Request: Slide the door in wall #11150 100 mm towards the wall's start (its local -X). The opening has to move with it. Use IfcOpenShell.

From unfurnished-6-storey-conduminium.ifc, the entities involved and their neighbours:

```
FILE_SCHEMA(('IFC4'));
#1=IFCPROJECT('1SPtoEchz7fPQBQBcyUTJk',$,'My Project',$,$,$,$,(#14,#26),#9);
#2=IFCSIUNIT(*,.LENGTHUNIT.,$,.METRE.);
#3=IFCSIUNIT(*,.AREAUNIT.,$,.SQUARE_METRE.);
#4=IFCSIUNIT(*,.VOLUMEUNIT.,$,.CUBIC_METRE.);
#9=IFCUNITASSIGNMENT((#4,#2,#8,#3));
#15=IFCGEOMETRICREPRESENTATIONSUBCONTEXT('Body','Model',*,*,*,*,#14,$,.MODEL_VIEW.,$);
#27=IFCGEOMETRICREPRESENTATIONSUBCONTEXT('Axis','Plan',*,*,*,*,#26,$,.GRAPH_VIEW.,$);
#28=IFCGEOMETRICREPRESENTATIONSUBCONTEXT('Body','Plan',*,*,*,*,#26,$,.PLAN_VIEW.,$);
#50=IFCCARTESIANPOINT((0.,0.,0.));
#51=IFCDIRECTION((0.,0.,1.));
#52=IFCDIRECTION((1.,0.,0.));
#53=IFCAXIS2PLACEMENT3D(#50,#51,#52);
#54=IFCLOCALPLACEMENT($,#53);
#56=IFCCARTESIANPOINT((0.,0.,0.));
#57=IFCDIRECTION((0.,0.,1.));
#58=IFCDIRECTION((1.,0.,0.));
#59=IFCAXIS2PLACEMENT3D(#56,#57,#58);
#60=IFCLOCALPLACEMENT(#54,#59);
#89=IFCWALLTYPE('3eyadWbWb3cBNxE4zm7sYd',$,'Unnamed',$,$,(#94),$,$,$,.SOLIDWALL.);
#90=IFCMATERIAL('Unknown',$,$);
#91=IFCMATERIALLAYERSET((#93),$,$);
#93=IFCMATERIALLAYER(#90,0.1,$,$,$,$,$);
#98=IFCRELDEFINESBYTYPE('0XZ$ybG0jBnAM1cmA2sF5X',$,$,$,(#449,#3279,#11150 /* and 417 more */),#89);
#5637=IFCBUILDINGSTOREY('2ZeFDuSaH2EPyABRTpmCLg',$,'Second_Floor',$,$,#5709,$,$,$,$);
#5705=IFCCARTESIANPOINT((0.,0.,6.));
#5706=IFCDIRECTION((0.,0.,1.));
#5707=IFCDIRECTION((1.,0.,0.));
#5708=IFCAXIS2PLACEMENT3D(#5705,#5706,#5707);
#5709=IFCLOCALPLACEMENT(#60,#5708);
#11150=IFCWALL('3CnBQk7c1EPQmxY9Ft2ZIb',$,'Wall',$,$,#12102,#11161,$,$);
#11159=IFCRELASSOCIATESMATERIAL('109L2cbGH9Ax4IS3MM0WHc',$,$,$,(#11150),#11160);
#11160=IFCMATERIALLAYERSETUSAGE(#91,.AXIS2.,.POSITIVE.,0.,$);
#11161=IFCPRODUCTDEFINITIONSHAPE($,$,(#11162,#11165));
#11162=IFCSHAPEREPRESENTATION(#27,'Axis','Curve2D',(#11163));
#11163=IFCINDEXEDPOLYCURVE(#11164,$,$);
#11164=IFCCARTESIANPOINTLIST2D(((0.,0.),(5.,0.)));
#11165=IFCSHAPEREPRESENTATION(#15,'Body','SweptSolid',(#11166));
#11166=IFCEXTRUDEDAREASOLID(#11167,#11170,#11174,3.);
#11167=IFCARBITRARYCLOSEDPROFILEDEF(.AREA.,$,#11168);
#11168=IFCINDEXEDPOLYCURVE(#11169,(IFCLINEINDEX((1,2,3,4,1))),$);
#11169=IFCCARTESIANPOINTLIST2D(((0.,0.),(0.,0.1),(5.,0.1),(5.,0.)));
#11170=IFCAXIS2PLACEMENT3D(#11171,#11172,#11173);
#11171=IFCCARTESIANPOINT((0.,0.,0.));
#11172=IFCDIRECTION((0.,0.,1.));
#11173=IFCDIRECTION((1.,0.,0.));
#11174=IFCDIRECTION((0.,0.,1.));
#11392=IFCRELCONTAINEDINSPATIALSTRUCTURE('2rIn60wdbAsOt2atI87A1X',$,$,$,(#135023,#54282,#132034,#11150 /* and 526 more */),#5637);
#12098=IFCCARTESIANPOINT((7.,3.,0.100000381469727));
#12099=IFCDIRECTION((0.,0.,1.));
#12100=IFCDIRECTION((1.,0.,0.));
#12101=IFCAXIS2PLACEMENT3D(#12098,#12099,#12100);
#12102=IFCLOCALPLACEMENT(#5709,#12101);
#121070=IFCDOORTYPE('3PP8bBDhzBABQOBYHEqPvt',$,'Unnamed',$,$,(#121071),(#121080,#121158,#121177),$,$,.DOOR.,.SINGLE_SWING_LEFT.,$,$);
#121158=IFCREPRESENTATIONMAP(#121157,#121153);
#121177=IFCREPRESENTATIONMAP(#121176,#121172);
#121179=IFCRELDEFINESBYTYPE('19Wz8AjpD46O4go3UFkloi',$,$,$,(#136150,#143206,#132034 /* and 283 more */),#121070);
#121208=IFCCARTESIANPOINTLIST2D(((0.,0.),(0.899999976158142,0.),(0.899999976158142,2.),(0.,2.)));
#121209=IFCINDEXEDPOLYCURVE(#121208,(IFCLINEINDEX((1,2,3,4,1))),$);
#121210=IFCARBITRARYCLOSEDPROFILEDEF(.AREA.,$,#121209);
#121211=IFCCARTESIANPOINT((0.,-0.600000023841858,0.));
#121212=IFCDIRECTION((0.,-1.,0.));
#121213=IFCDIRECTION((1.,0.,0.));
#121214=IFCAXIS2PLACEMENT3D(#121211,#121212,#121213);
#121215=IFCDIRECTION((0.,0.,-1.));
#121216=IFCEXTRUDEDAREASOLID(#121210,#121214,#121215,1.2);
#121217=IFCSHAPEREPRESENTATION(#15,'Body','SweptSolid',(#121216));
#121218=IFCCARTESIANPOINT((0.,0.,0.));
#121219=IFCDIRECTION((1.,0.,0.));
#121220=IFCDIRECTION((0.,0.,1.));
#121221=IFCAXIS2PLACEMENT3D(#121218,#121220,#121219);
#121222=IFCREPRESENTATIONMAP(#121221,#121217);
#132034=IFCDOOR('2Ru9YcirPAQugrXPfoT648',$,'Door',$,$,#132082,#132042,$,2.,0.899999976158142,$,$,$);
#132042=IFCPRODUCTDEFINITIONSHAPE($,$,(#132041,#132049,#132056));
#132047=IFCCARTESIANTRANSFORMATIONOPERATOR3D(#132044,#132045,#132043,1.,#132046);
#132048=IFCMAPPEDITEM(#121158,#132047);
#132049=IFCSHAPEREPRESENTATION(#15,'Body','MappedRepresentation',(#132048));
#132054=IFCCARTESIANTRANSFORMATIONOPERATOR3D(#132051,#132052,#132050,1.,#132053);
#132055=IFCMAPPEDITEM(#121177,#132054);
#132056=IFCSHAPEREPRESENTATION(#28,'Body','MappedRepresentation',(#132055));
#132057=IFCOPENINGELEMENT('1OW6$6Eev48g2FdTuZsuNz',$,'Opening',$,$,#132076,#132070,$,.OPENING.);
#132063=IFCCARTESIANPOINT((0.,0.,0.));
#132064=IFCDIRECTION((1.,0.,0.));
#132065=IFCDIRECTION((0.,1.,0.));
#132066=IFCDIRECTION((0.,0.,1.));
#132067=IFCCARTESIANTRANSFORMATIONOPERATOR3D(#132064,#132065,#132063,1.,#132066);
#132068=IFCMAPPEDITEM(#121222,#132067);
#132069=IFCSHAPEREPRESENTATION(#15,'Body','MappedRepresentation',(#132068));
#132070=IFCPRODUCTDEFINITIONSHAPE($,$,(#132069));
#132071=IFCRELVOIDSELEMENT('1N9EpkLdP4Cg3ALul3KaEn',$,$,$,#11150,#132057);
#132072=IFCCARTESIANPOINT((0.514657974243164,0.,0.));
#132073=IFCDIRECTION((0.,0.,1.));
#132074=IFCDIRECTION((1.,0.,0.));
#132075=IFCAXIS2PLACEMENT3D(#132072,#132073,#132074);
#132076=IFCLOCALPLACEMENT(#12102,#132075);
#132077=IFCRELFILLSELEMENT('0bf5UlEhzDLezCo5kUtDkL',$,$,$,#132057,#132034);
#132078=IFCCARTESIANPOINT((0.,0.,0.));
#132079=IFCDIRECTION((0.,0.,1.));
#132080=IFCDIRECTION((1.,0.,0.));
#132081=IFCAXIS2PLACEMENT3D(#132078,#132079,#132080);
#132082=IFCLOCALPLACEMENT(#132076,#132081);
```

```python
import ifcopenshell
import ifcopenshell.api.geometry
import ifcopenshell.util.placement
import ifcopenshell.util.unit

model = ifcopenshell.open("unfurnished-6-storey-conduminium.ifc")
unit_scale = ifcopenshell.util.unit.calculate_unit_scale(model)

door = model.by_id(132034)
opening = door.FillsVoids[0].RelatingOpeningElement
wall = opening.VoidsElements[0].RelatingBuildingElement

wall_matrix = ifcopenshell.util.placement.get_local_placement(wall.ObjectPlacement)
shift = wall_matrix[:3, 0] * -0.1 / unit_scale
before = ifcopenshell.util.placement.get_local_placement(door.ObjectPlacement)[:3, 3].copy()

# The door is placed relative to its opening, so it follows when the opening moves.
matrix = ifcopenshell.util.placement.get_local_placement(opening.ObjectPlacement)
matrix[:3, 3] += shift
ifcopenshell.api.geometry.edit_object_placement(
    model, product=opening, matrix=matrix, is_si=False, should_transform_children=True
)

after = ifcopenshell.util.placement.get_local_placement(door.ObjectPlacement)[:3, 3]
print("door moved by", (after - before).round(3) + 0.0)

model.write("unfurnished-6-storey-conduminium_edited.ifc")
```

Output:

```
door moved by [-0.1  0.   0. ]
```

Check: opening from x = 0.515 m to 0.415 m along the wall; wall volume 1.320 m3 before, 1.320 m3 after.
